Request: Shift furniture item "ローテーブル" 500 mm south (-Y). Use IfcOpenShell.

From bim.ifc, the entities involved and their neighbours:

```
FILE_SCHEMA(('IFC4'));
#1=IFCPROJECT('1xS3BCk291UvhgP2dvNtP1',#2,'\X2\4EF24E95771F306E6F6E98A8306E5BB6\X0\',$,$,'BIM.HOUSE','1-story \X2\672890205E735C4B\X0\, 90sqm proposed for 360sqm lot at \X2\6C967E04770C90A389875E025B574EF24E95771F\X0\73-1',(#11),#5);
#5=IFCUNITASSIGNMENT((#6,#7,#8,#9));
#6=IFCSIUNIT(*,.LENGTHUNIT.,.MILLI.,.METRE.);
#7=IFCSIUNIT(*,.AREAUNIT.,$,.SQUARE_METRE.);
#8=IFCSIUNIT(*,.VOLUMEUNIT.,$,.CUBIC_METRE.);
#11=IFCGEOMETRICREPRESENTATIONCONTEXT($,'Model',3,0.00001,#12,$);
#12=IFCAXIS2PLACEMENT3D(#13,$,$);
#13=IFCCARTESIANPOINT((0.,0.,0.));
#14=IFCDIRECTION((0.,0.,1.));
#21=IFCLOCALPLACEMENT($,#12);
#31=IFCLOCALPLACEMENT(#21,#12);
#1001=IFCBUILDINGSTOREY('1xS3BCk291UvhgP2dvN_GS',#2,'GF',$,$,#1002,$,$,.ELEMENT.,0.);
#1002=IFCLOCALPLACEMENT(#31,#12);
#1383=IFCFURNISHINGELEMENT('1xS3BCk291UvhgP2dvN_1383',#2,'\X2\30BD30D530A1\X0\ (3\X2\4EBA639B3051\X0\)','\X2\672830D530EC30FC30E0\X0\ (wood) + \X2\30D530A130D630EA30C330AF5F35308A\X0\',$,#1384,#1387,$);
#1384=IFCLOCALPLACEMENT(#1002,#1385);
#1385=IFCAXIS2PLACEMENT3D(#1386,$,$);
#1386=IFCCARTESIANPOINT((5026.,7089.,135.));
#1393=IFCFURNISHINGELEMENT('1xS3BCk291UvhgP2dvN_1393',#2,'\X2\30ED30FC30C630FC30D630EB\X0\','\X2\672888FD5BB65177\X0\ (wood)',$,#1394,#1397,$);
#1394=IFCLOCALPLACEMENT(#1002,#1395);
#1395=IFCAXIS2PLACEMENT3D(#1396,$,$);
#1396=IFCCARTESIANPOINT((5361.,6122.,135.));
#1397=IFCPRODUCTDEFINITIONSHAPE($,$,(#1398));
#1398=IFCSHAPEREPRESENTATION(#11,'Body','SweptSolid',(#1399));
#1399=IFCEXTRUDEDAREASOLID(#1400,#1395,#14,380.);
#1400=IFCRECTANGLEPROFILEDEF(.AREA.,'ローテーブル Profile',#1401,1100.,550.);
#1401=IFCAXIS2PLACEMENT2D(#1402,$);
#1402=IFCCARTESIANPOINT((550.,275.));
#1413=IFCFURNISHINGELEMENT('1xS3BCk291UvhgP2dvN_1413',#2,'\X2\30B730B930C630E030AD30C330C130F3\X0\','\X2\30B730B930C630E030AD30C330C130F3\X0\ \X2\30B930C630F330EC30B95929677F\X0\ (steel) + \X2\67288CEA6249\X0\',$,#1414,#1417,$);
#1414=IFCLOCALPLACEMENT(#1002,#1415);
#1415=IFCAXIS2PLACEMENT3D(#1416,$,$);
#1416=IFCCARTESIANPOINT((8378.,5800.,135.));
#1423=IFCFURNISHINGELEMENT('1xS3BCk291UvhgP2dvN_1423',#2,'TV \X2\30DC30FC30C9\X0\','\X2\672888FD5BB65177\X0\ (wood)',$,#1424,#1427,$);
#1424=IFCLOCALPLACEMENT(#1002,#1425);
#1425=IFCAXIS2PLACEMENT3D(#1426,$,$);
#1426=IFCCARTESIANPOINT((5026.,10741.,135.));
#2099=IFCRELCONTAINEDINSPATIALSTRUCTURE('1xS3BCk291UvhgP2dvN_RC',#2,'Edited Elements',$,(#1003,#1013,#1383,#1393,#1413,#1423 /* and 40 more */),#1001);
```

```python
import ifcopenshell
import ifcopenshell.api.geometry
import ifcopenshell.util.placement
import ifcopenshell.util.unit

model = ifcopenshell.open("bim.ifc")
unit_scale = ifcopenshell.util.unit.calculate_unit_scale(model)

item = model.by_guid("1xS3BCk291UvhgP2dvN_1393")
matrix = ifcopenshell.util.placement.get_local_placement(item.ObjectPlacement)
matrix[1, 3] -= 0.5 / unit_scale
ifcopenshell.api.geometry.edit_object_placement(model, product=item, matrix=matrix, is_si=False)

print(ifcopenshell.util.placement.get_local_placement(item.ObjectPlacement).round(3) + 0.0)

model.write("bim_updated.ifc")
```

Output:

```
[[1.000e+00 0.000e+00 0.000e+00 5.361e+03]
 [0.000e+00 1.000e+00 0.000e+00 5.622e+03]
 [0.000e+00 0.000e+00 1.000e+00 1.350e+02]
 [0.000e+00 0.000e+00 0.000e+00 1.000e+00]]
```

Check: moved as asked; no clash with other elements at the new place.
